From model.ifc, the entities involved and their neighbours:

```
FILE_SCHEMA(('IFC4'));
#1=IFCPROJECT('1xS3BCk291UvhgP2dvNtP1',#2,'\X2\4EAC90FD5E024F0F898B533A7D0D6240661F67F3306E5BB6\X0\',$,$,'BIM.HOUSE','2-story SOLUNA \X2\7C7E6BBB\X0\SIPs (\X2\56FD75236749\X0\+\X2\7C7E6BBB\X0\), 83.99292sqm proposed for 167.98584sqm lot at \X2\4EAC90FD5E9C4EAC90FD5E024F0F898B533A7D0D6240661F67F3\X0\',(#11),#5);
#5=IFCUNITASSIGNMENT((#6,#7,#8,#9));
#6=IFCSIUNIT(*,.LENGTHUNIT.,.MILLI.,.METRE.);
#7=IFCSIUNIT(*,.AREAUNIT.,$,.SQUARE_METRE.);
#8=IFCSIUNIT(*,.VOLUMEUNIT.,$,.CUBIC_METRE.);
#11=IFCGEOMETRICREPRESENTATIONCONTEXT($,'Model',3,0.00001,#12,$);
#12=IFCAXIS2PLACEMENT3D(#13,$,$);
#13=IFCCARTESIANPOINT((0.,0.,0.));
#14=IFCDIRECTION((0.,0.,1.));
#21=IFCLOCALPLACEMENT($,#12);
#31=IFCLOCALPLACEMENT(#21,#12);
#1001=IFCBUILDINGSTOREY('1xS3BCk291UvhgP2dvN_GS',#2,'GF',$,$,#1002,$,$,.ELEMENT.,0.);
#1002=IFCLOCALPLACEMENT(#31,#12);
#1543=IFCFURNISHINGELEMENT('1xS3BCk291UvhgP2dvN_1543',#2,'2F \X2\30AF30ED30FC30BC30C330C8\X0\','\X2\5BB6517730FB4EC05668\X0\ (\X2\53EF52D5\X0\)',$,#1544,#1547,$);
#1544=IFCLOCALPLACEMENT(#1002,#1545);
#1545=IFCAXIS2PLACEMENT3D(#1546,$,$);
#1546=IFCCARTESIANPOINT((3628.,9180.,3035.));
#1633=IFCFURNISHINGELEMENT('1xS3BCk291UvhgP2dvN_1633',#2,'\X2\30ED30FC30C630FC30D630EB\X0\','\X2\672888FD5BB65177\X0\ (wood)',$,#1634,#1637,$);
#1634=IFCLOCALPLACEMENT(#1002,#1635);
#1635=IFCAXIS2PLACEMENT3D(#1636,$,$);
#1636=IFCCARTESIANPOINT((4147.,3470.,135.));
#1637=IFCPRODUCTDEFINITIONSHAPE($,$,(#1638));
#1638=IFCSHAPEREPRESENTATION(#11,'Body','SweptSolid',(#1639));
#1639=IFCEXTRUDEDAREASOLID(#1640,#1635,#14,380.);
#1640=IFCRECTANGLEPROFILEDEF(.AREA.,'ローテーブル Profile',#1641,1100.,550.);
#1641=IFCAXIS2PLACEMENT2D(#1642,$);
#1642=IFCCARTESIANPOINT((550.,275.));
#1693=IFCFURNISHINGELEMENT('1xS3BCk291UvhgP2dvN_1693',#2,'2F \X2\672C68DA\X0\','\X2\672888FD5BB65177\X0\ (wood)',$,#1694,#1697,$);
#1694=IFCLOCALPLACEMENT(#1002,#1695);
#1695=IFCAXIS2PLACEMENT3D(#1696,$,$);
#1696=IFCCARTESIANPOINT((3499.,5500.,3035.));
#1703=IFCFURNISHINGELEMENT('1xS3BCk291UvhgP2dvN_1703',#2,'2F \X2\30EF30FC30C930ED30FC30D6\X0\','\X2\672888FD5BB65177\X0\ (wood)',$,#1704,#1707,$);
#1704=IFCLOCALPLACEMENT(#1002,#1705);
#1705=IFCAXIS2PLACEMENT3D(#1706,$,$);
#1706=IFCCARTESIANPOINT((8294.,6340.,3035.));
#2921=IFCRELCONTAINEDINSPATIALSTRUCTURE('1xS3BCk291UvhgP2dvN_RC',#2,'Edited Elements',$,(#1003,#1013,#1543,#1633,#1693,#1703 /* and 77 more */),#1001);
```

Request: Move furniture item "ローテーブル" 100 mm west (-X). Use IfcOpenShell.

```python
import ifcopenshell
import ifcopenshell.api.geometry
import ifcopenshell.util.placement
import ifcopenshell.util.unit

model = ifcopenshell.open("model.ifc")
unit_scale = ifcopenshell.util.unit.calculate_unit_scale(model)

item = model.by_guid("1xS3BCk291UvhgP2dvN_1633")
matrix = ifcopenshell.util.placement.get_local_placement(item.ObjectPlacement)
matrix[0, 3] -= 0.1 / unit_scale
ifcopenshell.api.geometry.edit_object_placement(model, product=item, matrix=matrix, is_si=False)

print(ifcopenshell.util.placement.get_local_placement(item.ObjectPlacement).round(3) + 0.0)

model.write("model_edited.ifc")
```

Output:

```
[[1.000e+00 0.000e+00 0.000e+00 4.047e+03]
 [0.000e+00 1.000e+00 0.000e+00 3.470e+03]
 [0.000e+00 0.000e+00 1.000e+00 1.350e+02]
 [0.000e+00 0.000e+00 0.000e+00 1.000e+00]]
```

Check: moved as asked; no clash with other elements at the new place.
